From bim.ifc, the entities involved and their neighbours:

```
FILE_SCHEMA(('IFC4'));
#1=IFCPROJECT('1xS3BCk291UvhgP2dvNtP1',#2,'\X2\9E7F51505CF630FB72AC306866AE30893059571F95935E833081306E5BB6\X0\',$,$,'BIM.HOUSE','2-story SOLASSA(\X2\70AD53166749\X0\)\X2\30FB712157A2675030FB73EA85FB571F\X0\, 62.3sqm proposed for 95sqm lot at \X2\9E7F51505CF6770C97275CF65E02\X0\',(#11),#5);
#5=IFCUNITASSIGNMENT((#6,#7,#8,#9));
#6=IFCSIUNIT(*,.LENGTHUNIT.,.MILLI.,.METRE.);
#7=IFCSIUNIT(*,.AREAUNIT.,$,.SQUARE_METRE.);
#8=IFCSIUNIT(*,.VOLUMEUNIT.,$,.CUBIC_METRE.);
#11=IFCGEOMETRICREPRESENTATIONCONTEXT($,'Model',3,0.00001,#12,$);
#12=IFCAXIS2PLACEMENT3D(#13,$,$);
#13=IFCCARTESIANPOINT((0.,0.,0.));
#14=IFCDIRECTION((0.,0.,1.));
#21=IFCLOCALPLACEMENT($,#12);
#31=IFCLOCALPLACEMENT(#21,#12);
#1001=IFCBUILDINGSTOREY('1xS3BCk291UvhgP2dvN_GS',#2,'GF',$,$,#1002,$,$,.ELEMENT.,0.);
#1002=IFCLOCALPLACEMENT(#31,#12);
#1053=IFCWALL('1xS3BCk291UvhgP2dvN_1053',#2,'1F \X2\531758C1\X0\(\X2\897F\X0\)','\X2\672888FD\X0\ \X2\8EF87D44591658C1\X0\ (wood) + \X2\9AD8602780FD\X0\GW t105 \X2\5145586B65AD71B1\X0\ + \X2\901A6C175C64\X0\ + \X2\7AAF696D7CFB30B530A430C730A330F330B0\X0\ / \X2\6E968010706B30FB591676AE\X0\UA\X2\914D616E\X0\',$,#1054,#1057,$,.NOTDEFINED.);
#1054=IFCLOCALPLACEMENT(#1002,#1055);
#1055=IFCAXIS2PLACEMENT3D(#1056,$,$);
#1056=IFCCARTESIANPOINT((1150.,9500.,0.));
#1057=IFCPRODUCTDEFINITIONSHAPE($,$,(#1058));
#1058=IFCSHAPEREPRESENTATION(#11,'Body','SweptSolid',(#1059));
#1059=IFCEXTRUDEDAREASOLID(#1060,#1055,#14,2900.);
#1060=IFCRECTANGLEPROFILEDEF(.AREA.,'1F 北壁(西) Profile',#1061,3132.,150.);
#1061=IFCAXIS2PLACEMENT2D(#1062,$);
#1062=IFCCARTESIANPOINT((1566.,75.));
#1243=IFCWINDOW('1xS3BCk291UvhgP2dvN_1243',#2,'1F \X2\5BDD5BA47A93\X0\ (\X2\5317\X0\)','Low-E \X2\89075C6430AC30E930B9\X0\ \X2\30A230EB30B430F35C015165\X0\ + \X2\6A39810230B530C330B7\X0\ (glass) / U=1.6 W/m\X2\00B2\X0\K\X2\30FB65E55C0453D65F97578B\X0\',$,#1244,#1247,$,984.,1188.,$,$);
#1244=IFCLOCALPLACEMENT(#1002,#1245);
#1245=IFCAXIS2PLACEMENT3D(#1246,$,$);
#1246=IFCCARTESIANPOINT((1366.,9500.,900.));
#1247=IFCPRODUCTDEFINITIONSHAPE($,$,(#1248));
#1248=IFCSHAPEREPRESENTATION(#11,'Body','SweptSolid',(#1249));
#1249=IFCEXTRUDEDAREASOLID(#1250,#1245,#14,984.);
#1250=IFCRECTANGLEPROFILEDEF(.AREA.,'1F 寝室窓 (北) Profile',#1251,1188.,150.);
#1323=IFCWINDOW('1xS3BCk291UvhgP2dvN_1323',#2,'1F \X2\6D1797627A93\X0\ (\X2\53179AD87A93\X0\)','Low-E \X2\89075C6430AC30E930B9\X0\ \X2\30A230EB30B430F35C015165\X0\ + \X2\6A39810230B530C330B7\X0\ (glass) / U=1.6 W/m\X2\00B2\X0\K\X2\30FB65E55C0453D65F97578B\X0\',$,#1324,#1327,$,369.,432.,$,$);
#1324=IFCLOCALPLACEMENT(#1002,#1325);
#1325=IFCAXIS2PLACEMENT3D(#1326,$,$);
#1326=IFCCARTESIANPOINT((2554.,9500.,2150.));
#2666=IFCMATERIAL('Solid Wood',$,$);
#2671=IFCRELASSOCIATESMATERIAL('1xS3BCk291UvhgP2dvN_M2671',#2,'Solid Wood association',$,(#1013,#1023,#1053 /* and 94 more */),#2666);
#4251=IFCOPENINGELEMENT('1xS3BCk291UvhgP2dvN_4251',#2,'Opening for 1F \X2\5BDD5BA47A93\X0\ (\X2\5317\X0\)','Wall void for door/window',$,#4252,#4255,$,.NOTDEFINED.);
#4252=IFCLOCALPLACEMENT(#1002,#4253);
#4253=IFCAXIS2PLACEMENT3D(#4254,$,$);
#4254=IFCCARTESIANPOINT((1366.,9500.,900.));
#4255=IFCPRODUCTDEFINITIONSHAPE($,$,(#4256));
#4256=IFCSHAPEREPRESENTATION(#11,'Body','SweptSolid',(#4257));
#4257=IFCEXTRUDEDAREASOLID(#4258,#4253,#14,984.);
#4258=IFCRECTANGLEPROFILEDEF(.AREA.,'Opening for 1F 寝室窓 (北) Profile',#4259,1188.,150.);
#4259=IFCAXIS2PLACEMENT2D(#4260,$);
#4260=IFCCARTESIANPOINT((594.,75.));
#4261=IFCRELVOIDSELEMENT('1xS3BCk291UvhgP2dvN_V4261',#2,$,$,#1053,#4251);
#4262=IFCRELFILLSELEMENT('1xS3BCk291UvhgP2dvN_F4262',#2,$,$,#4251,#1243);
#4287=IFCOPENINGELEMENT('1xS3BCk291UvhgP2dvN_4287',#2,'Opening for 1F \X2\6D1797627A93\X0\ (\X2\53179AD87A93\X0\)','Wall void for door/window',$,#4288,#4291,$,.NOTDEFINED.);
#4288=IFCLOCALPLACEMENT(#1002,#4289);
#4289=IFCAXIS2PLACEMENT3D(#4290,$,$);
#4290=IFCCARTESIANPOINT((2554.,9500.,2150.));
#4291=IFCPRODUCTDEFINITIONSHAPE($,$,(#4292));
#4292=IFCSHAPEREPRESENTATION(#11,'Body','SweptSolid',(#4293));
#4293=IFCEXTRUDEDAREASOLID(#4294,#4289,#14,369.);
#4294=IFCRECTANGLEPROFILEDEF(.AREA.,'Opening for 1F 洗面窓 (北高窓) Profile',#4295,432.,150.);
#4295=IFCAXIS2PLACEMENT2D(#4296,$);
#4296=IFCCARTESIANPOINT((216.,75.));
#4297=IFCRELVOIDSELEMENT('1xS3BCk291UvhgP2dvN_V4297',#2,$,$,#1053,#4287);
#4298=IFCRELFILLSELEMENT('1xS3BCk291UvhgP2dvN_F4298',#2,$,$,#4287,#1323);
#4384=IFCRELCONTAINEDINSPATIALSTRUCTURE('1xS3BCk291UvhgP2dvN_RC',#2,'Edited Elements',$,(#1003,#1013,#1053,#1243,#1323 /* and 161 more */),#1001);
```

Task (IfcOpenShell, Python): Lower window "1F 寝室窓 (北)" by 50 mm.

```python
import numpy as np
import ifcopenshell
import ifcopenshell.api.geometry
import ifcopenshell.util.placement
import ifcopenshell.util.unit

model = ifcopenshell.open("bim.ifc")
unit_scale = ifcopenshell.util.unit.calculate_unit_scale(model)

window = model.by_guid("1xS3BCk291UvhgP2dvN_1243")
opening = window.FillsVoids[0].RelatingOpeningElement
dz = -50.0

shift = np.array([0.0, 0.0, dz])
# The window is not placed relative to its opening, so move both.
for product in (opening, window):
    matrix = ifcopenshell.util.placement.get_local_placement(product.ObjectPlacement)
    matrix[:3, 3] += shift
    ifcopenshell.api.geometry.edit_object_placement(model, product=product, matrix=matrix, is_si=False)

print(f"moved by {dz * unit_scale:+.3f} m")

model.write("bim_rev.ifc")
```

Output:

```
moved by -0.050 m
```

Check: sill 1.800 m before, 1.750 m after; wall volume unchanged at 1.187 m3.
